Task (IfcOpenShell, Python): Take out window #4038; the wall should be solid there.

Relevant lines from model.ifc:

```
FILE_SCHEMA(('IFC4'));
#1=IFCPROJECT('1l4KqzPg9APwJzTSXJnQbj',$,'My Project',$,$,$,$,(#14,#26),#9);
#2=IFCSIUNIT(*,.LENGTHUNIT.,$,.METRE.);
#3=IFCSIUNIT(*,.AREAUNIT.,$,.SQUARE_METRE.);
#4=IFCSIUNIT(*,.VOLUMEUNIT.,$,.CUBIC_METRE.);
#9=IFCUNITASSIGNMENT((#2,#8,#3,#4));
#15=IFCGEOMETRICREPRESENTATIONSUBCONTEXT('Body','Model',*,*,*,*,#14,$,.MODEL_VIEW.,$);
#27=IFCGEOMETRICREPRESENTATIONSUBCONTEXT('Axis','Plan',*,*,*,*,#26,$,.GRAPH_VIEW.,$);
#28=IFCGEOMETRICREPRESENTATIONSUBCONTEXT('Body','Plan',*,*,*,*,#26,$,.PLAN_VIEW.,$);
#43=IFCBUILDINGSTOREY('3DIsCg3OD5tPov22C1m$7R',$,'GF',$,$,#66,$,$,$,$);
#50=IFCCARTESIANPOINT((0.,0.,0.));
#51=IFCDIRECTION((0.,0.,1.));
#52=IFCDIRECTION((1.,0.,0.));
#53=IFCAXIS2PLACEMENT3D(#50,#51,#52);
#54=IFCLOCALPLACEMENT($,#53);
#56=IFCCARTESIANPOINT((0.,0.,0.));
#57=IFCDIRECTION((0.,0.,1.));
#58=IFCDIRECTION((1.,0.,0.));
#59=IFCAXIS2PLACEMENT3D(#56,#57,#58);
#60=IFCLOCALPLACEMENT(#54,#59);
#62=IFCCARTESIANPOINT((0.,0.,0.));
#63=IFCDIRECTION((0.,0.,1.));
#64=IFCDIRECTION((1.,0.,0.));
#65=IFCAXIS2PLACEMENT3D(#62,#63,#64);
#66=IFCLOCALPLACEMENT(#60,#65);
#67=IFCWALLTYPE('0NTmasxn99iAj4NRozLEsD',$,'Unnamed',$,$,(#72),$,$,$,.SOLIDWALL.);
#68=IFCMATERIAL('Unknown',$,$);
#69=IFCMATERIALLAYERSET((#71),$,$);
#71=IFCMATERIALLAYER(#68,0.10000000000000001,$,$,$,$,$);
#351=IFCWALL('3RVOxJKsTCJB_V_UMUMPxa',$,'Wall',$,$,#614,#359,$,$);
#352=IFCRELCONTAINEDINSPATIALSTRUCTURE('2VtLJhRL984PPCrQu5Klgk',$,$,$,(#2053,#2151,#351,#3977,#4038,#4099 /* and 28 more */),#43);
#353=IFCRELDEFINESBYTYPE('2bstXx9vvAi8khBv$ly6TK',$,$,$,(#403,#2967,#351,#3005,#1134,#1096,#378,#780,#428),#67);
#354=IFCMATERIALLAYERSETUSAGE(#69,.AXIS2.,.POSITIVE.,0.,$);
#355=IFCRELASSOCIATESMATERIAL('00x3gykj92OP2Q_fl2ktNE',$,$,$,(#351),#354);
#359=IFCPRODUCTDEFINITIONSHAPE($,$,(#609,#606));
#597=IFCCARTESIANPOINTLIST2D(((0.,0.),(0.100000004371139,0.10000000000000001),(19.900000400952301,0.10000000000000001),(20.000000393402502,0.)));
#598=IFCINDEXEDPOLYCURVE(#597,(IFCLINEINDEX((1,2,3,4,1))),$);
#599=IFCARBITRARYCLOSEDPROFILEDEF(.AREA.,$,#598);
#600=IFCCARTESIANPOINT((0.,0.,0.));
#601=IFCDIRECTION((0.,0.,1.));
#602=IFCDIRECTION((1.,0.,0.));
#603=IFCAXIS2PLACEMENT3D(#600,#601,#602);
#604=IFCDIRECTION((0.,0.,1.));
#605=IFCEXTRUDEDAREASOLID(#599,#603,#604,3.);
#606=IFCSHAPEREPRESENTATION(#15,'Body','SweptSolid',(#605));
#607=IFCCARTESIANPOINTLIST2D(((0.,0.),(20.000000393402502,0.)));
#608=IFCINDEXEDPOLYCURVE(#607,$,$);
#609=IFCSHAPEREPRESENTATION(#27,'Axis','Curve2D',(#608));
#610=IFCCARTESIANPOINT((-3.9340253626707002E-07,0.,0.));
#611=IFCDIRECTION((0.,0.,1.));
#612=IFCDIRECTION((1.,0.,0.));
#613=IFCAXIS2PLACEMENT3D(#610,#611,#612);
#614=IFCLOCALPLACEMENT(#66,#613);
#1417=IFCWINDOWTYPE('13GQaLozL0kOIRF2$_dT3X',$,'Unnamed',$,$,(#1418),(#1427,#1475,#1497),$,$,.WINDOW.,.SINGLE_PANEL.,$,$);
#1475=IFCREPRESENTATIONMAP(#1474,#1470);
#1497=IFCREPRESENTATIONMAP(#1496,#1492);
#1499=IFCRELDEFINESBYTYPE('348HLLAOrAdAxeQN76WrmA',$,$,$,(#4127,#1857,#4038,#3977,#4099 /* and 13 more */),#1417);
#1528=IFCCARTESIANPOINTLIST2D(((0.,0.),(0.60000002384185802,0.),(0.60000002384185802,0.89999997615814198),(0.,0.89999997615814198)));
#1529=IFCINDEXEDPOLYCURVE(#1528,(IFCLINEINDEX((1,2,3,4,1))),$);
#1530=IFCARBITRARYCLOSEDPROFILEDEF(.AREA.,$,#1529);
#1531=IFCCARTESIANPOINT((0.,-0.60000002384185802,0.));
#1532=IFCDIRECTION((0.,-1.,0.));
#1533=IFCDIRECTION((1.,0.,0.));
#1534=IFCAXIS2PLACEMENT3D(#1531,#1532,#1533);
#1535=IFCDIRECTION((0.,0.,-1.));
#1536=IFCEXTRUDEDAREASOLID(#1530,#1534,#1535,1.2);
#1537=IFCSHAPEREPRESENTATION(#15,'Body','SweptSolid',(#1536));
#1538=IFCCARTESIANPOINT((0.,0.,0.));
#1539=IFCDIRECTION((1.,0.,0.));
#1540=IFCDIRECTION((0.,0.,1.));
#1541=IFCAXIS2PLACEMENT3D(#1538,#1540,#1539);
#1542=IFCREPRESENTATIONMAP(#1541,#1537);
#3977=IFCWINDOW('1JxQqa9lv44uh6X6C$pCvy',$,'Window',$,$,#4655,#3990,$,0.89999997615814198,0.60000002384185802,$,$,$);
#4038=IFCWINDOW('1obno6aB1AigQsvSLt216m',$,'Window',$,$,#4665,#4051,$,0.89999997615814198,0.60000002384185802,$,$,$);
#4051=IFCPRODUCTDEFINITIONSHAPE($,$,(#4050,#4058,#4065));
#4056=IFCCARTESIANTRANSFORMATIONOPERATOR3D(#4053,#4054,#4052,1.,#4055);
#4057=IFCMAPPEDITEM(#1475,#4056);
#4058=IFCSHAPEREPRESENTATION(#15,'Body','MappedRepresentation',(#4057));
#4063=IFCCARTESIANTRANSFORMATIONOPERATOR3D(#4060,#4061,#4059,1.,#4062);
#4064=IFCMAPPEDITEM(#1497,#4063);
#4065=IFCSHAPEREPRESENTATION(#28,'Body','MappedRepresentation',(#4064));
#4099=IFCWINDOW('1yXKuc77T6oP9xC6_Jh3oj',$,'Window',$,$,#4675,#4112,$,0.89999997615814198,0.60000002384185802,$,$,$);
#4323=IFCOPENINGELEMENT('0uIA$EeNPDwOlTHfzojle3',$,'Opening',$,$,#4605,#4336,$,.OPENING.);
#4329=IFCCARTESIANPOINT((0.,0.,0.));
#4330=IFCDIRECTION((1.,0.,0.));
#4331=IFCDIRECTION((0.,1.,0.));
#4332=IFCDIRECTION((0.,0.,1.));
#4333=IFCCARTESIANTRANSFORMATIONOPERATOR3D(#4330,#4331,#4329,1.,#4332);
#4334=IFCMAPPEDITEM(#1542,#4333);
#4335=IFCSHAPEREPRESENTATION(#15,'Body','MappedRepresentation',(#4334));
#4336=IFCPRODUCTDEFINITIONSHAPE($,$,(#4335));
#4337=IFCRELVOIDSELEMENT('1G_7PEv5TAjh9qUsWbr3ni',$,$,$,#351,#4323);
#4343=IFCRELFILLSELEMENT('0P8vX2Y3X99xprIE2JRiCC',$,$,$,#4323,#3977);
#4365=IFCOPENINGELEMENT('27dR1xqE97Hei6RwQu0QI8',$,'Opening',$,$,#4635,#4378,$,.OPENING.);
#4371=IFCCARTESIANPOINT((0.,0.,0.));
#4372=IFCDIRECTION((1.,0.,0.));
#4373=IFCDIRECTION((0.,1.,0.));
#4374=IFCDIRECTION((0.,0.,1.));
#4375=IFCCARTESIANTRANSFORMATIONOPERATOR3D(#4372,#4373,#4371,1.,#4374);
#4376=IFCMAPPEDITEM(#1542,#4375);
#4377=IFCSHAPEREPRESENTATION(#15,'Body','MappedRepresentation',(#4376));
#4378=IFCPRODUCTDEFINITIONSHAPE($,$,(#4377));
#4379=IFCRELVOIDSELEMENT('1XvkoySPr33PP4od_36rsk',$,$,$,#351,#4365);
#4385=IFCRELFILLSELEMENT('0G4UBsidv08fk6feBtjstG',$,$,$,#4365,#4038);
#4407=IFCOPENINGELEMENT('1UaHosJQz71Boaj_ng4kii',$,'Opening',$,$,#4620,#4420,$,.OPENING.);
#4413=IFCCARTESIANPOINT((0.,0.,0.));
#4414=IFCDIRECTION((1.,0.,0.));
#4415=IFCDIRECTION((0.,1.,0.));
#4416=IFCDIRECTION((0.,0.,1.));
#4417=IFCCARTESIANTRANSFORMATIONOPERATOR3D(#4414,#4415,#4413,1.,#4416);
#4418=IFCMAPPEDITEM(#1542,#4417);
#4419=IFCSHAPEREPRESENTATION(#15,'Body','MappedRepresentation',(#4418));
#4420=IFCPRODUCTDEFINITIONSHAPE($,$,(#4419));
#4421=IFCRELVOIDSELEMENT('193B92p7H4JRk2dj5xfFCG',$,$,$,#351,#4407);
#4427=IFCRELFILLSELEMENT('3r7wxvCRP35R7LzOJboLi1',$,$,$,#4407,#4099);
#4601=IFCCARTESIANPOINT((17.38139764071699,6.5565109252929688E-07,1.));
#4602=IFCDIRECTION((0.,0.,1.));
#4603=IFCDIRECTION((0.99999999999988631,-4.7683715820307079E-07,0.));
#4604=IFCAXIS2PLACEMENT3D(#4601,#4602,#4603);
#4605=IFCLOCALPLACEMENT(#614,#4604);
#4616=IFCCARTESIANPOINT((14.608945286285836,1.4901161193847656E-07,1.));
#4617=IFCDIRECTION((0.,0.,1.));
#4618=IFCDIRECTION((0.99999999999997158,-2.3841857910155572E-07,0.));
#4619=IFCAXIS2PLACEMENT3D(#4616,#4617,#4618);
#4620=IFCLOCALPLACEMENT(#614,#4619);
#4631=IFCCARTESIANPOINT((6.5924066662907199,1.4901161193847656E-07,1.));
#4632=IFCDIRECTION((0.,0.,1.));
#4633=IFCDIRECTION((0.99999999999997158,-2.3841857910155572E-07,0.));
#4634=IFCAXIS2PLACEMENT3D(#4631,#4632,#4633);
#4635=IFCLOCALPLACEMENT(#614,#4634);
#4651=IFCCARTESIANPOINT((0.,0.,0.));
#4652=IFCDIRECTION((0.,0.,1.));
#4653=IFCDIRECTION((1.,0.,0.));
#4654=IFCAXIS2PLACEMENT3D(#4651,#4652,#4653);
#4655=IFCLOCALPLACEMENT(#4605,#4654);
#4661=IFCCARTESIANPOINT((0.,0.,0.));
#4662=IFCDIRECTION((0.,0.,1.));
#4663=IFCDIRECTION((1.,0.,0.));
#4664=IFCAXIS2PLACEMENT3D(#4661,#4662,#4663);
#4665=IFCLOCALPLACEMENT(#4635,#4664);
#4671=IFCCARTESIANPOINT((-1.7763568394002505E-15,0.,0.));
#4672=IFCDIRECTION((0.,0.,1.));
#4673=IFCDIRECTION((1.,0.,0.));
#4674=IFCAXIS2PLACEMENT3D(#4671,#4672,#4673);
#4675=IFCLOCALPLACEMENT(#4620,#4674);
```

```python
import ifcopenshell
import ifcopenshell.api.feature
import ifcopenshell.api.root
import ifcopenshell.geom
import ifcopenshell.util.shape

model = ifcopenshell.open("model.ifc")
settings = ifcopenshell.geom.settings()


def volume(element):
    """Net volume in cubic metres, openings subtracted."""
    shape = ifcopenshell.geom.create_shape(settings, element)
    return ifcopenshell.util.shape.get_volume(shape.geometry)


window = model.by_guid("1obno6aB1AigQsvSLt216m")
opening = window.FillsVoids[0].RelatingOpeningElement
wall = opening.VoidsElements[0].RelatingBuildingElement
before = volume(wall)

ifcopenshell.api.root.remove_product(model, product=window)
ifcopenshell.api.feature.remove_feature(model, feature=opening)

after = volume(wall)

print(f"wall volume {before:.3f} -> {after:.3f} m3")

model.write("model_v2.ifc")
```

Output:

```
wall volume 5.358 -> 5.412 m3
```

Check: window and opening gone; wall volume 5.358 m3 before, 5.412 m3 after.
